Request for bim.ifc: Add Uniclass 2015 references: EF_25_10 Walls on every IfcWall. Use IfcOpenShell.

First a look at what the model holds.

```python
import ifcopenshell

model = ifcopenshell.open("bim.ifc")
print(model.schema)
print("classifications:", [c.Name for c in model.by_type("IfcClassification")])
for ifc_class in ("IfcDoor", "IfcRoof", "IfcStair", "IfcWall", "IfcWindow"):
    print(ifc_class, len(model.by_type(ifc_class)))
```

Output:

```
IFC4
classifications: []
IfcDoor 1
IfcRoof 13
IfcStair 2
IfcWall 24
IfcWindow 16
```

```python
import ifcopenshell
import ifcopenshell.api.classification

model = ifcopenshell.open("bim.ifc")

system = ifcopenshell.api.classification.add_classification(model, classification="Uniclass 2015")

codes = {
    "IfcWall": ("EF_25_10", "Walls"),
}
for ifc_class, (code, name) in codes.items():
    products = model.by_type(ifc_class)
    ifcopenshell.api.classification.add_reference(
        model, products=products, classification=system, identification=code, name=name
    )
    print(code, len(products))

model.write("bim-out.ifc")
```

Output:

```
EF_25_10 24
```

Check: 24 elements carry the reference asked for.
